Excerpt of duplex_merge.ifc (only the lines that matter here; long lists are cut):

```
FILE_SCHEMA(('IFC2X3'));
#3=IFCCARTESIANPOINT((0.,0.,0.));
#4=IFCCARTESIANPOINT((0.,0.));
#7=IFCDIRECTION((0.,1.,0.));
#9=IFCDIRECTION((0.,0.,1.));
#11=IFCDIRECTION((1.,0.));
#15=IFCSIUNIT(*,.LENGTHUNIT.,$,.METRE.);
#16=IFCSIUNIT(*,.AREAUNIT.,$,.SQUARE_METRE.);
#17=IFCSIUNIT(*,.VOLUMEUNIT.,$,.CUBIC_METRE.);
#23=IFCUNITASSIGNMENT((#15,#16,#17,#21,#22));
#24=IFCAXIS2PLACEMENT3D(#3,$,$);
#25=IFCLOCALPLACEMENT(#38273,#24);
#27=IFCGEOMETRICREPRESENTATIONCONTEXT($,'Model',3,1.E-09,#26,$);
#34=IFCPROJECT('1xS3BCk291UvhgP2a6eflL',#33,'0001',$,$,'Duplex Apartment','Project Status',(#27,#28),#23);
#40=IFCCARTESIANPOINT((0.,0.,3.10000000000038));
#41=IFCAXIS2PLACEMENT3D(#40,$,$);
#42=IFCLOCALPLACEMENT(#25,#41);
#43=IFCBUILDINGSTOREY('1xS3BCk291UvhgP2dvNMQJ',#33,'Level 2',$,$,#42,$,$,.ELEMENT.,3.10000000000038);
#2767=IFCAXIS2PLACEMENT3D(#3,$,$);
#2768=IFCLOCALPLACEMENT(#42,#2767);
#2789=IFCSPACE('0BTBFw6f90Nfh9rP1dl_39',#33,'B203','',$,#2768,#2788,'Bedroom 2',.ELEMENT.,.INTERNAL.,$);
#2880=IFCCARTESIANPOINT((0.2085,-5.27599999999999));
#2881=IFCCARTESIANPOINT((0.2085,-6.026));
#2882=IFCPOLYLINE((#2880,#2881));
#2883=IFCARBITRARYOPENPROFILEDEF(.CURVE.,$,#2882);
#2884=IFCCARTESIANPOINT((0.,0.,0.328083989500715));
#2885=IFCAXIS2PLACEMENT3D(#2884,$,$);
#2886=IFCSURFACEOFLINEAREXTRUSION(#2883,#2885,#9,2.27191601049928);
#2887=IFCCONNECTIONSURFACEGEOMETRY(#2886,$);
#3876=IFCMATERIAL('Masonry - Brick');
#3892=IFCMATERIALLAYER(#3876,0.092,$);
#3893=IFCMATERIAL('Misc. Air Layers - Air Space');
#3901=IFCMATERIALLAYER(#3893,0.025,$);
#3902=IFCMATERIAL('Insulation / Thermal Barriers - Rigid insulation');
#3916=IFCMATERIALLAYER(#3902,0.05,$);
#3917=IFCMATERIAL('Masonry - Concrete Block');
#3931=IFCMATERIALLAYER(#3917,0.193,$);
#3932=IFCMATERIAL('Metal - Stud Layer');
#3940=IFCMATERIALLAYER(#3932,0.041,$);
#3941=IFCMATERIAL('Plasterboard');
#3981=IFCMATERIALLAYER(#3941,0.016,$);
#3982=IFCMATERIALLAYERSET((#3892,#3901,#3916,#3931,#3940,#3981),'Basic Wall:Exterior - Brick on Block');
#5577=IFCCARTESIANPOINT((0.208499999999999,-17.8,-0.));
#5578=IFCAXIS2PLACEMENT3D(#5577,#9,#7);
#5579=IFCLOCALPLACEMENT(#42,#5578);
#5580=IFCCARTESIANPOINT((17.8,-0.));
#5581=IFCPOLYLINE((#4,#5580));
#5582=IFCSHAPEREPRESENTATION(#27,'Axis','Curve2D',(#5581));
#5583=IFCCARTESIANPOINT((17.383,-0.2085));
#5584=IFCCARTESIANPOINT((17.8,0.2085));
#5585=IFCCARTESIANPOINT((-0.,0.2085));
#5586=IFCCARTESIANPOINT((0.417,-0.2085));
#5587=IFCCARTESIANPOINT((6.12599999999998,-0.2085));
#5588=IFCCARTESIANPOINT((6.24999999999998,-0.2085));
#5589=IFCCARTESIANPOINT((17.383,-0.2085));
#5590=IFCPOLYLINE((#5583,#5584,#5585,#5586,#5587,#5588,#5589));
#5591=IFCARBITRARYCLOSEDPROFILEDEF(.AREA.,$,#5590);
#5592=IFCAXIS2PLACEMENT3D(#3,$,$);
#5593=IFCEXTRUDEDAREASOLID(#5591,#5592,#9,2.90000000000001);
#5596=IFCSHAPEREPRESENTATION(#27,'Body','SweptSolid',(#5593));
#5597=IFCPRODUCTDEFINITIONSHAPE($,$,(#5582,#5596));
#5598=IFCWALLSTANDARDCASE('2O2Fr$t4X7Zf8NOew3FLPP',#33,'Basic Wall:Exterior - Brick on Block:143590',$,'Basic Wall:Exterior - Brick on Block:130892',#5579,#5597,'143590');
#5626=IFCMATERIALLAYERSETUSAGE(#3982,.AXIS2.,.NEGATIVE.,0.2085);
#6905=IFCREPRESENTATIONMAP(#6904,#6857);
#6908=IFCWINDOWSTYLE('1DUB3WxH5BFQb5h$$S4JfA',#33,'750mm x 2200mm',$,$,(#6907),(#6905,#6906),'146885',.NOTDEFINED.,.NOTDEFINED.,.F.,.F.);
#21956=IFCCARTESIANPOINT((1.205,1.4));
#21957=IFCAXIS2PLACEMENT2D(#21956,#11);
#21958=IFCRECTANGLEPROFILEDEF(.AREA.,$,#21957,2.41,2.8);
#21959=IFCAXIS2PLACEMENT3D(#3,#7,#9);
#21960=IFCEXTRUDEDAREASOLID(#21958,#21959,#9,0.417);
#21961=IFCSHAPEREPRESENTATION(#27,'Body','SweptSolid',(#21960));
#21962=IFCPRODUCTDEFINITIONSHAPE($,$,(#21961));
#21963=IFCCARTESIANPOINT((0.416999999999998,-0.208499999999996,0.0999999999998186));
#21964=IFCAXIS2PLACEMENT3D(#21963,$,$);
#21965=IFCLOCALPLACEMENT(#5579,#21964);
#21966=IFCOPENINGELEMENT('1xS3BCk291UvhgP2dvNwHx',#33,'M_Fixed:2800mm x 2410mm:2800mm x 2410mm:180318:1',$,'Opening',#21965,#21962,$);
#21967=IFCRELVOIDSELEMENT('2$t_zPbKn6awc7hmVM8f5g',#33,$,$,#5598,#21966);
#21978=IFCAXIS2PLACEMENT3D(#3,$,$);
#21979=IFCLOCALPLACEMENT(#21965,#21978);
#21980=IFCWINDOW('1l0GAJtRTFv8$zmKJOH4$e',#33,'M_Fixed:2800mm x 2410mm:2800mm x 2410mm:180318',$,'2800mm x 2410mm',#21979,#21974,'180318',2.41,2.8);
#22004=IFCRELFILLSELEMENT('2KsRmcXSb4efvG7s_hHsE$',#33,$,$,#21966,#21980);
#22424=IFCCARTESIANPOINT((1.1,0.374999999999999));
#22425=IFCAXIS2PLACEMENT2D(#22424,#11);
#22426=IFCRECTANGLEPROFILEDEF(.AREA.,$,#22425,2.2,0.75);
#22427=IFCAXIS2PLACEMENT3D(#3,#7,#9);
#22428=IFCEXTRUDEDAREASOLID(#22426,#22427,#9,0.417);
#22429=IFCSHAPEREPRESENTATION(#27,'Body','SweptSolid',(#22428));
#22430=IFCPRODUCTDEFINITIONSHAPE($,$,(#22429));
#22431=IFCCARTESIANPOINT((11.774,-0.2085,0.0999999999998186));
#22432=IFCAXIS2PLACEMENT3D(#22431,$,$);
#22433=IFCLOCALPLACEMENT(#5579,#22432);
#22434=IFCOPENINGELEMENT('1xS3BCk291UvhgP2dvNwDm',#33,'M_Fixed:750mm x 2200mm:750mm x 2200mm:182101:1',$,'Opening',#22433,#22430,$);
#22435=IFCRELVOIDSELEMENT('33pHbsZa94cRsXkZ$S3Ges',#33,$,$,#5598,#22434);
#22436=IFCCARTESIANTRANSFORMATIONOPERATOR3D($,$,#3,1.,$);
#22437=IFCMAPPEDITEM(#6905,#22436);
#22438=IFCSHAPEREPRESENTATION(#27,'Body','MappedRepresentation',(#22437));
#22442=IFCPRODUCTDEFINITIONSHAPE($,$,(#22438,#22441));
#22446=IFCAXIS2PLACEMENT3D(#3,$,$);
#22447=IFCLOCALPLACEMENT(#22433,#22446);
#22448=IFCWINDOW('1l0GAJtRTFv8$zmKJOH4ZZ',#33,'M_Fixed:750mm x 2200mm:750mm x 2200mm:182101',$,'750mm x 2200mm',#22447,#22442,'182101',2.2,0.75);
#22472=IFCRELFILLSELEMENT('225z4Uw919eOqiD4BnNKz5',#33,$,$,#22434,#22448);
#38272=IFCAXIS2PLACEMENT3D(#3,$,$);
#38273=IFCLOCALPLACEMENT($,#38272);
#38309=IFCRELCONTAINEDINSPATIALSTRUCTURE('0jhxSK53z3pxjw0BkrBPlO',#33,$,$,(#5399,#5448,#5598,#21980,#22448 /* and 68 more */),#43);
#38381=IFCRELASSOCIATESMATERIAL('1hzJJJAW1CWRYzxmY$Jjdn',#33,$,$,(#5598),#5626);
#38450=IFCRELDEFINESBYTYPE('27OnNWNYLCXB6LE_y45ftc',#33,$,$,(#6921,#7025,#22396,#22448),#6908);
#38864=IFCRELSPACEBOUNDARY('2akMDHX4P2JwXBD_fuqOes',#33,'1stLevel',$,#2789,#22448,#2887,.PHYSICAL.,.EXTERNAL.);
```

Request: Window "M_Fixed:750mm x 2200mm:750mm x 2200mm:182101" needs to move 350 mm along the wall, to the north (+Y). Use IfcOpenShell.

```python
import numpy as np
import ifcopenshell
import ifcopenshell.api.geometry
import ifcopenshell.util.placement
import ifcopenshell.util.unit

model = ifcopenshell.open("duplex_merge.ifc")
unit_scale = ifcopenshell.util.unit.calculate_unit_scale(model)

window = model.by_guid("1l0GAJtRTFv8$zmKJOH4ZZ")
opening = window.FillsVoids[0].RelatingOpeningElement
wall = opening.VoidsElements[0].RelatingBuildingElement

wall_matrix = ifcopenshell.util.placement.get_local_placement(wall.ObjectPlacement)
shift = wall_matrix[:3, 0] * 0.35 / unit_scale
before = ifcopenshell.util.placement.get_local_placement(window.ObjectPlacement)[:3, 3].copy()

# The window is placed relative to its opening, so it follows when the opening moves.
matrix = ifcopenshell.util.placement.get_local_placement(opening.ObjectPlacement)
matrix[:3, 3] += shift
ifcopenshell.api.geometry.edit_object_placement(
    model, product=opening, matrix=matrix, is_si=False, should_transform_children=True
)

# Space boundary surfaces are stored in each space's coordinates; move them too.
for rel in window.ProvidesBoundaries:
    if not rel.ConnectionGeometry:
        continue
    surface = rel.ConnectionGeometry.SurfaceOnRelatingElement
    space_matrix = ifcopenshell.util.placement.get_local_placement(rel.RelatingSpace.ObjectPlacement)
    point = np.array(surface.Position.Location.Coordinates) + space_matrix[:3, :3].T @ shift
    surface.Position = model.createIfcAxis2Placement3D(
        model.createIfcCartesianPoint(point.tolist()), surface.Position.Axis, surface.Position.RefDirection
    )

after = ifcopenshell.util.placement.get_local_placement(window.ObjectPlacement)[:3, 3]
print("window moved by", (after - before).round(3) + 0.0)

model.write("duplex_merge_rev.ifc")
```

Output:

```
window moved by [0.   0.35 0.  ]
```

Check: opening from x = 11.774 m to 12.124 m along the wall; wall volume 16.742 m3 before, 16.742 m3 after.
